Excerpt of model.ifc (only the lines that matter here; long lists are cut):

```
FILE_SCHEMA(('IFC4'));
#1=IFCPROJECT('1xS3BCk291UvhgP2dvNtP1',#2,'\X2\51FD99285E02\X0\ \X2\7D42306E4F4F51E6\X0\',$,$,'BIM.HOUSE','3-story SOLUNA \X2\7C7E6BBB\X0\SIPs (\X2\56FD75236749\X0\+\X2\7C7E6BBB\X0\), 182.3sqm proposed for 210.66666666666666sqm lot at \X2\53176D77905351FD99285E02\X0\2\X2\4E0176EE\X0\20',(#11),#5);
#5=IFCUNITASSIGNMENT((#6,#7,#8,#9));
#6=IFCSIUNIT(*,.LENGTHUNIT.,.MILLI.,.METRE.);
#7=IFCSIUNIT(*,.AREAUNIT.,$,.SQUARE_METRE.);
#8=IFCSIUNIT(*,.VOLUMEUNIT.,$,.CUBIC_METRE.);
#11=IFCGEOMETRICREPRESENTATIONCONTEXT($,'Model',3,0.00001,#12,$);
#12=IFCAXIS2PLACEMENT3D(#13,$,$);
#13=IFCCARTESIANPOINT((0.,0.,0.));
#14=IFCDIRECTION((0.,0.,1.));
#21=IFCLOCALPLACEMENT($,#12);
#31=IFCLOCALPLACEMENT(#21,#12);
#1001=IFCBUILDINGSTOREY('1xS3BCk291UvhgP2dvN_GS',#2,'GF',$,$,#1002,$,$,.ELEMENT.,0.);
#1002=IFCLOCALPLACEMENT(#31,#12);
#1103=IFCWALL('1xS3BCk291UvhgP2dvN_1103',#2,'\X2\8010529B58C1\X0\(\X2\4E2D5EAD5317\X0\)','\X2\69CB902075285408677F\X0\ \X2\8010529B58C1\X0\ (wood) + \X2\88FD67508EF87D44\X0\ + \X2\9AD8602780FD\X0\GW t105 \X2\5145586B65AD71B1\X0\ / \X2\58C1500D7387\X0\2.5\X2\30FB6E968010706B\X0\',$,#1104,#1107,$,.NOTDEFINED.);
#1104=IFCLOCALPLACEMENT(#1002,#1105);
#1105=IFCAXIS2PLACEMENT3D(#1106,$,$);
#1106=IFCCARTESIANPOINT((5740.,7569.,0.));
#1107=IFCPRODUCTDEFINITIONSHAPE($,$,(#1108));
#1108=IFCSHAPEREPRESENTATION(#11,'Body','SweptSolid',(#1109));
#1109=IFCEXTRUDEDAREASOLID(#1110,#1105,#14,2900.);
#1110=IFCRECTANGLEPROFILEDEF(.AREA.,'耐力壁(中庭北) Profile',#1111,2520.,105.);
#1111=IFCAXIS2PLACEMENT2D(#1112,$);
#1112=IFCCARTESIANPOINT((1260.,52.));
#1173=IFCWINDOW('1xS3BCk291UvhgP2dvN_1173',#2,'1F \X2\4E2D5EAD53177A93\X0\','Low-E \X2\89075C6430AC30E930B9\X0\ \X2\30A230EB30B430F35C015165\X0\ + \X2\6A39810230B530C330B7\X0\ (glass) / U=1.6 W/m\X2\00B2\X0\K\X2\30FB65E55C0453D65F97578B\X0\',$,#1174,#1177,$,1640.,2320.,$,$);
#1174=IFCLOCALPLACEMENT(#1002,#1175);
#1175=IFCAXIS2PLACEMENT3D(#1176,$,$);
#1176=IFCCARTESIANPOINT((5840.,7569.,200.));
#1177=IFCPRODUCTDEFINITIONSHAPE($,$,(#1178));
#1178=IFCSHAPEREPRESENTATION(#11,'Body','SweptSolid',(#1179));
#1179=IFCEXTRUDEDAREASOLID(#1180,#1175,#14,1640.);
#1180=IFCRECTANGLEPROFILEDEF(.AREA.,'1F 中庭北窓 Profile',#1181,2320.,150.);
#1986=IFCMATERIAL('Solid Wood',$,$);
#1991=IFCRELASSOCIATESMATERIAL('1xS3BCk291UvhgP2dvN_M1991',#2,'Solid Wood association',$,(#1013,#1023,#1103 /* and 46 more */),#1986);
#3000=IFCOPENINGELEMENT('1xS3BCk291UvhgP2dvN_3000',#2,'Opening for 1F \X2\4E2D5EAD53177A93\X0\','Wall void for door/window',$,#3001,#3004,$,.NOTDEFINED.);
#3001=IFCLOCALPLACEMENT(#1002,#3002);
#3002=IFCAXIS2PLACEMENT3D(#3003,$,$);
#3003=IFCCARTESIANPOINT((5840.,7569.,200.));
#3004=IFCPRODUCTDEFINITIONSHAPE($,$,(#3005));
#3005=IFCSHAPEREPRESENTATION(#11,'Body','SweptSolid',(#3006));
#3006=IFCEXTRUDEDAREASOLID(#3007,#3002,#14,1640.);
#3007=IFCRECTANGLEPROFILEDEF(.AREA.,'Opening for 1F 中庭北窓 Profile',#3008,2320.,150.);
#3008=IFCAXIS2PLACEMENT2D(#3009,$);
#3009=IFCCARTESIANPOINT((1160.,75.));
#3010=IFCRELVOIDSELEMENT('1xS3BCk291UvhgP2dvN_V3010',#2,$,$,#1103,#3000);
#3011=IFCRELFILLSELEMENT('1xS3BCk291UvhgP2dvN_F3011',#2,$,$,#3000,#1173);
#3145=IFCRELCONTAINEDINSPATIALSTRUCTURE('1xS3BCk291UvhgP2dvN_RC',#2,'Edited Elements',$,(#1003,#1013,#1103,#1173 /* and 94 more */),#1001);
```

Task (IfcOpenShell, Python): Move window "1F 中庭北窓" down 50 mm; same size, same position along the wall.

```python
import numpy as np
import ifcopenshell
import ifcopenshell.api.geometry
import ifcopenshell.util.placement
import ifcopenshell.util.unit

model = ifcopenshell.open("model.ifc")
unit_scale = ifcopenshell.util.unit.calculate_unit_scale(model)

window = model.by_guid("1xS3BCk291UvhgP2dvN_1173")
opening = window.FillsVoids[0].RelatingOpeningElement
dz = -50.0

shift = np.array([0.0, 0.0, dz])
# The window is not placed relative to its opening, so move both.
for product in (opening, window):
    matrix = ifcopenshell.util.placement.get_local_placement(product.ObjectPlacement)
    matrix[:3, 3] += shift
    ifcopenshell.api.geometry.edit_object_placement(model, product=product, matrix=matrix, is_si=False)

print(f"moved by {dz * unit_scale:+.3f} m")

model.write("model-out.ifc")
```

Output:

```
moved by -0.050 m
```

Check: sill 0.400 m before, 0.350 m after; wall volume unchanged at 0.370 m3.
